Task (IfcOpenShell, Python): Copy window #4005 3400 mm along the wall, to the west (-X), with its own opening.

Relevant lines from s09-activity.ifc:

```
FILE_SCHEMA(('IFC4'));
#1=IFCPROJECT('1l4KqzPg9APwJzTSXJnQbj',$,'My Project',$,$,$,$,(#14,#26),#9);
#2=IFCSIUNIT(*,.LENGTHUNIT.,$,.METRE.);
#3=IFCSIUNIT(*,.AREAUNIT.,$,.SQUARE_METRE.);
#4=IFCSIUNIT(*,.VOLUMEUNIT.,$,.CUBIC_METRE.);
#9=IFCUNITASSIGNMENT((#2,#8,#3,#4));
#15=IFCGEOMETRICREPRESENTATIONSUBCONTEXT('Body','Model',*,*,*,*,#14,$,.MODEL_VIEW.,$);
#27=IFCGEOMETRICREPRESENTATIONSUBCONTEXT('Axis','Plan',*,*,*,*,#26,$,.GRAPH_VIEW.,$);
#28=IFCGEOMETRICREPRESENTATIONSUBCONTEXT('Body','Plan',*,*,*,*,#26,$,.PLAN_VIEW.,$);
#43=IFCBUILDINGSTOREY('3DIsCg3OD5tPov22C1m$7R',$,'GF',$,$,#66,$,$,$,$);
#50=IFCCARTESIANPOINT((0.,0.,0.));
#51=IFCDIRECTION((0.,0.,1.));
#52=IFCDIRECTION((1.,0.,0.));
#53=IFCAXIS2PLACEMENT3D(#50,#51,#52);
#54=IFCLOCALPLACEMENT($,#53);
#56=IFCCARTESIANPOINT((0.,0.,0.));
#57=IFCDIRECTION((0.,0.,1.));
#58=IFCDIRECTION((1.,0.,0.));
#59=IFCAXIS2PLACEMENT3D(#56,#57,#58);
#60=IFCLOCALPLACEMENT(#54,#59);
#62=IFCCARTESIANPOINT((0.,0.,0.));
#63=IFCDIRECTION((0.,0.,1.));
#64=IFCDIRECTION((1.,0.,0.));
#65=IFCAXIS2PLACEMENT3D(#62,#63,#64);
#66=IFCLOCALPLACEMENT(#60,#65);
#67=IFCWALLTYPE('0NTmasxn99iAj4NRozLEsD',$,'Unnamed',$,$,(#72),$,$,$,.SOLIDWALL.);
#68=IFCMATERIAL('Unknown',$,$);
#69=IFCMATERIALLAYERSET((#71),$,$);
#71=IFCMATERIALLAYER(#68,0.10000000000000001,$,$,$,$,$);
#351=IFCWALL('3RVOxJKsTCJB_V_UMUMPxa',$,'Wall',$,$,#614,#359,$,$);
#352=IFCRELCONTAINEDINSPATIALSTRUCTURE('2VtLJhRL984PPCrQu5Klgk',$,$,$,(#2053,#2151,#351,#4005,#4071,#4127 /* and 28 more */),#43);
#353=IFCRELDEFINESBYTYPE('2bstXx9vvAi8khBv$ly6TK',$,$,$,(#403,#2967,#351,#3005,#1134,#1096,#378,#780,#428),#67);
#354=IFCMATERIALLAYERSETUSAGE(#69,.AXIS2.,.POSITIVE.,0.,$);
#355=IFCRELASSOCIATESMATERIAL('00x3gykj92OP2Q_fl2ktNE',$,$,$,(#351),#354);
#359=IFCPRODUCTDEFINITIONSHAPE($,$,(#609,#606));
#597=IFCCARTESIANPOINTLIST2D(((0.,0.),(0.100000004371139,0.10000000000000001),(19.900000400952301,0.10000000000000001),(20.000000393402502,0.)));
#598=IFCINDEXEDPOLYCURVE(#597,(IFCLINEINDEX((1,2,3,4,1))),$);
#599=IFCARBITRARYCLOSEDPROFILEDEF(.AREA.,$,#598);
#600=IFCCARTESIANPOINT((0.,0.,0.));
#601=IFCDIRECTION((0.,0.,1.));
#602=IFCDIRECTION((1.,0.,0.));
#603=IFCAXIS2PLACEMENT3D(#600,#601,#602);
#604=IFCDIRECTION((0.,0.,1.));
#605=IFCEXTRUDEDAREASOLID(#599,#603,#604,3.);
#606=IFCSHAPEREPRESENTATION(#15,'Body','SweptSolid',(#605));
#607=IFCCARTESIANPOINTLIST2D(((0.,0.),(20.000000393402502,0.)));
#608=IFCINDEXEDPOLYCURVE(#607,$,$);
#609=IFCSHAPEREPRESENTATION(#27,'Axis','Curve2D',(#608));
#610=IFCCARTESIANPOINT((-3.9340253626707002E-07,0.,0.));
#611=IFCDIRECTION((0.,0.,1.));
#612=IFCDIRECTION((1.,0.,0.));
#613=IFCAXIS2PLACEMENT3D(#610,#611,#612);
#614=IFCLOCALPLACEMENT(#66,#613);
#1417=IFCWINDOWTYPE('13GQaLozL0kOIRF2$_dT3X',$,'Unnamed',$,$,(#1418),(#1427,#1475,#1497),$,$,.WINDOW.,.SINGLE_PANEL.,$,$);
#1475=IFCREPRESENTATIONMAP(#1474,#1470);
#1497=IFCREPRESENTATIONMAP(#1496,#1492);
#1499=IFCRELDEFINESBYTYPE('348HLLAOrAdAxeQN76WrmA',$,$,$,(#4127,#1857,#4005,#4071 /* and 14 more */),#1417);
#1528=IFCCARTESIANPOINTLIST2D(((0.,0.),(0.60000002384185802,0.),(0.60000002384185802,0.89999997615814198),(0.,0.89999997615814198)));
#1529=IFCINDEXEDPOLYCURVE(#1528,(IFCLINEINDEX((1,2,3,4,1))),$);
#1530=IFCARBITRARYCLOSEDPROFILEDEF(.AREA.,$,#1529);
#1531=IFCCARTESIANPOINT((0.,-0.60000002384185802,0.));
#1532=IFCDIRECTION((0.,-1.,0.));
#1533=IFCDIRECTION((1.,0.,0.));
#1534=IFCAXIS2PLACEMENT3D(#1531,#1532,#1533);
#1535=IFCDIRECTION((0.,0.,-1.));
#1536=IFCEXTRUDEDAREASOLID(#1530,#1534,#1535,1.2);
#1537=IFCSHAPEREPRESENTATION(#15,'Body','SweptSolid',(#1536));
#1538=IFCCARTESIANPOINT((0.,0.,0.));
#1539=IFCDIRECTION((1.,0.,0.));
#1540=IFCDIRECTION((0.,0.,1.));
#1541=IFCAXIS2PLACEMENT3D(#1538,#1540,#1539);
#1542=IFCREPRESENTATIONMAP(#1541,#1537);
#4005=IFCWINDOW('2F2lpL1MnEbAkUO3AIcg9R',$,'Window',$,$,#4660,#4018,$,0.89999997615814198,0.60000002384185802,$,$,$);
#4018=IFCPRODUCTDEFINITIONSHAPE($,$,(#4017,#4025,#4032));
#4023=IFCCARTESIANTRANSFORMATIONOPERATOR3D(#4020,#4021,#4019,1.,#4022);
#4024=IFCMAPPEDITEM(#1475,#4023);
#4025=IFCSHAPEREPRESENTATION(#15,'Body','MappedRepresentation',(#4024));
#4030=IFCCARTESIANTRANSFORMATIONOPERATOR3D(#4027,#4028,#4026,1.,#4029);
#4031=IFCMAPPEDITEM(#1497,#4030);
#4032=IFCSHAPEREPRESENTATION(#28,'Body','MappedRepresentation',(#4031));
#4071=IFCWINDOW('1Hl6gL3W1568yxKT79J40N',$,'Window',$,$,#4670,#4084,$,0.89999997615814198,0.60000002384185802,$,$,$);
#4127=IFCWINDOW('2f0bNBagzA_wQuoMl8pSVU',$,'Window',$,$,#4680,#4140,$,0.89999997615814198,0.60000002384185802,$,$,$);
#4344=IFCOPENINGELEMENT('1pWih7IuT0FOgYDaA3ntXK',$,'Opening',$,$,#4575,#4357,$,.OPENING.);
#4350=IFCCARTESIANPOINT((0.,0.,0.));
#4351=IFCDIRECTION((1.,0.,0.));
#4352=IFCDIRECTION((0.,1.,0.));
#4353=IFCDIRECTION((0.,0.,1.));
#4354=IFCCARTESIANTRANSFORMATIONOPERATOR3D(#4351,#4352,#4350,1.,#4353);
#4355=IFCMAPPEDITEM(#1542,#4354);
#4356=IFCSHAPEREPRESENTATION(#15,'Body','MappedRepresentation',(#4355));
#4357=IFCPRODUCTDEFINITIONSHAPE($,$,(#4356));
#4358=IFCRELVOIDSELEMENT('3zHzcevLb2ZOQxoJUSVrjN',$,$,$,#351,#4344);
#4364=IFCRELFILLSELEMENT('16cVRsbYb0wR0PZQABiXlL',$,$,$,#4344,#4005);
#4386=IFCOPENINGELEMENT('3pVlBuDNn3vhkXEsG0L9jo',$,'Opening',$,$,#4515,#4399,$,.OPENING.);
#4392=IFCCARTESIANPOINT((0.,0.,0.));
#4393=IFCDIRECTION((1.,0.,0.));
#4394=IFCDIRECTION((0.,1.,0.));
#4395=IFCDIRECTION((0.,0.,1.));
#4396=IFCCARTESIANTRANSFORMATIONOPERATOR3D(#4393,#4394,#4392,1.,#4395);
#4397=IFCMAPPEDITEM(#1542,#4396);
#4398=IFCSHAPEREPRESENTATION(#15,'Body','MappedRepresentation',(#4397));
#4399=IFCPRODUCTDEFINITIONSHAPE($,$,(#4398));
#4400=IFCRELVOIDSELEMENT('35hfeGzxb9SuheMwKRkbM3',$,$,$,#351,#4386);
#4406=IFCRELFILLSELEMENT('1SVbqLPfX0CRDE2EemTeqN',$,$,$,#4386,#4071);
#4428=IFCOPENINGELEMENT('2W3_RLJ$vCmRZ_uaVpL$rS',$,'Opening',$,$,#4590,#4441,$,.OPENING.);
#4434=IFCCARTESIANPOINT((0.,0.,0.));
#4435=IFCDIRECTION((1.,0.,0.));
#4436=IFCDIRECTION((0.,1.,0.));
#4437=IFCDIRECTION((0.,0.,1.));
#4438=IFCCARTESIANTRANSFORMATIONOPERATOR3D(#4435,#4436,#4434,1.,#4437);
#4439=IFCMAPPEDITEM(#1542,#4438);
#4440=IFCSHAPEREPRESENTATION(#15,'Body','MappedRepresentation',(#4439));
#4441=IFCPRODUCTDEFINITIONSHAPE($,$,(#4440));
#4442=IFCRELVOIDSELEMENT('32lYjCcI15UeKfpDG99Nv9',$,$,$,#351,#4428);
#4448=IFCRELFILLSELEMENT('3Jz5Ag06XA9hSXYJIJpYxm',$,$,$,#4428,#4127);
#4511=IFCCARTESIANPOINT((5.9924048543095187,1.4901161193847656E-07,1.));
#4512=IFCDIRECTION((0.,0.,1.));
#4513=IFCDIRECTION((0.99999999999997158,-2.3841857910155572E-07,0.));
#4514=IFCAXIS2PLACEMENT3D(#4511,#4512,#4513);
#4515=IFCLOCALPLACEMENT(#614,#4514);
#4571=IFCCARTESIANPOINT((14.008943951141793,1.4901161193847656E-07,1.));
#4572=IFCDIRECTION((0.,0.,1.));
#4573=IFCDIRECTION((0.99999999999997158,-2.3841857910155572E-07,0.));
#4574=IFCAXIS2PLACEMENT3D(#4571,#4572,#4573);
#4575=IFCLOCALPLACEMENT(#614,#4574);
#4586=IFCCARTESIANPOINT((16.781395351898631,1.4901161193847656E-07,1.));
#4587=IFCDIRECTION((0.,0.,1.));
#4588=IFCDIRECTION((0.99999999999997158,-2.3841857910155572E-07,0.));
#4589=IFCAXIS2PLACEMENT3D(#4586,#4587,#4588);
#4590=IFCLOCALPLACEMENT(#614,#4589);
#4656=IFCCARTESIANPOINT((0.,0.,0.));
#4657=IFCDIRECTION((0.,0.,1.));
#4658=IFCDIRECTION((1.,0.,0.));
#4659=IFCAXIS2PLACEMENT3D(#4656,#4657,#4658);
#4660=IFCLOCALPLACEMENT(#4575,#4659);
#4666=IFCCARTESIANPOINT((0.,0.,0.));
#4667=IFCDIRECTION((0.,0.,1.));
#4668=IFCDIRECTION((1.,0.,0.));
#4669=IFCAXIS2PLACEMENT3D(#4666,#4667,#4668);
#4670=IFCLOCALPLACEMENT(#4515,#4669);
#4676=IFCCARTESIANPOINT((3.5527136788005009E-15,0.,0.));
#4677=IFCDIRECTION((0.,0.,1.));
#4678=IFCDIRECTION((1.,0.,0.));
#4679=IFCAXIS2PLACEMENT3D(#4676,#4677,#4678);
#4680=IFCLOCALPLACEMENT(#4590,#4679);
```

```python
import ifcopenshell
import ifcopenshell.api.feature
import ifcopenshell.api.geometry
import ifcopenshell.api.root
import ifcopenshell.geom
import ifcopenshell.util.element
import ifcopenshell.util.placement
import ifcopenshell.util.shape

model = ifcopenshell.open("s09-activity.ifc")
settings = ifcopenshell.geom.settings()


def volume(element):
    """Net volume in cubic metres, openings subtracted."""
    shape = ifcopenshell.geom.create_shape(settings, element)
    return ifcopenshell.util.shape.get_volume(shape.geometry)


window = model.by_guid("2F2lpL1MnEbAkUO3AIcg9R")
opening = window.FillsVoids[0].RelatingOpeningElement
wall = opening.VoidsElements[0].RelatingBuildingElement
before = volume(wall)
shift = ifcopenshell.util.placement.get_local_placement(wall.ObjectPlacement)[:3, 0] * -3.4

# copy_class copies the void relationship, type, container and properties, but no geometry.
new_opening = ifcopenshell.api.root.copy_class(model, product=opening)
new_opening.Representation = ifcopenshell.util.element.copy_deep(
    model, opening.Representation, exclude=["IfcGeometricRepresentationContext", "IfcRepresentationMap"]
)
new_window = ifcopenshell.api.root.copy_class(model, product=window)
new_window.Representation = ifcopenshell.util.element.copy_deep(
    model, window.Representation, exclude=["IfcGeometricRepresentationContext", "IfcRepresentationMap"]
)
ifcopenshell.api.feature.add_filling(model, opening=new_opening, element=new_window)

for old, new in ((opening, new_opening), (window, new_window)):
    matrix = ifcopenshell.util.placement.get_local_placement(old.ObjectPlacement)
    matrix[:3, 3] += shift
    ifcopenshell.api.geometry.edit_object_placement(model, product=new, matrix=matrix, is_si=False)

after = volume(wall)

print(f"wall volume {before:.3f} -> {after:.3f} m3")

model.write("s09-activity_updated.ifc")
```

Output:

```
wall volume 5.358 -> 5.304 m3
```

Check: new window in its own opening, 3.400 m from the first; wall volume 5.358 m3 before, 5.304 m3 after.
